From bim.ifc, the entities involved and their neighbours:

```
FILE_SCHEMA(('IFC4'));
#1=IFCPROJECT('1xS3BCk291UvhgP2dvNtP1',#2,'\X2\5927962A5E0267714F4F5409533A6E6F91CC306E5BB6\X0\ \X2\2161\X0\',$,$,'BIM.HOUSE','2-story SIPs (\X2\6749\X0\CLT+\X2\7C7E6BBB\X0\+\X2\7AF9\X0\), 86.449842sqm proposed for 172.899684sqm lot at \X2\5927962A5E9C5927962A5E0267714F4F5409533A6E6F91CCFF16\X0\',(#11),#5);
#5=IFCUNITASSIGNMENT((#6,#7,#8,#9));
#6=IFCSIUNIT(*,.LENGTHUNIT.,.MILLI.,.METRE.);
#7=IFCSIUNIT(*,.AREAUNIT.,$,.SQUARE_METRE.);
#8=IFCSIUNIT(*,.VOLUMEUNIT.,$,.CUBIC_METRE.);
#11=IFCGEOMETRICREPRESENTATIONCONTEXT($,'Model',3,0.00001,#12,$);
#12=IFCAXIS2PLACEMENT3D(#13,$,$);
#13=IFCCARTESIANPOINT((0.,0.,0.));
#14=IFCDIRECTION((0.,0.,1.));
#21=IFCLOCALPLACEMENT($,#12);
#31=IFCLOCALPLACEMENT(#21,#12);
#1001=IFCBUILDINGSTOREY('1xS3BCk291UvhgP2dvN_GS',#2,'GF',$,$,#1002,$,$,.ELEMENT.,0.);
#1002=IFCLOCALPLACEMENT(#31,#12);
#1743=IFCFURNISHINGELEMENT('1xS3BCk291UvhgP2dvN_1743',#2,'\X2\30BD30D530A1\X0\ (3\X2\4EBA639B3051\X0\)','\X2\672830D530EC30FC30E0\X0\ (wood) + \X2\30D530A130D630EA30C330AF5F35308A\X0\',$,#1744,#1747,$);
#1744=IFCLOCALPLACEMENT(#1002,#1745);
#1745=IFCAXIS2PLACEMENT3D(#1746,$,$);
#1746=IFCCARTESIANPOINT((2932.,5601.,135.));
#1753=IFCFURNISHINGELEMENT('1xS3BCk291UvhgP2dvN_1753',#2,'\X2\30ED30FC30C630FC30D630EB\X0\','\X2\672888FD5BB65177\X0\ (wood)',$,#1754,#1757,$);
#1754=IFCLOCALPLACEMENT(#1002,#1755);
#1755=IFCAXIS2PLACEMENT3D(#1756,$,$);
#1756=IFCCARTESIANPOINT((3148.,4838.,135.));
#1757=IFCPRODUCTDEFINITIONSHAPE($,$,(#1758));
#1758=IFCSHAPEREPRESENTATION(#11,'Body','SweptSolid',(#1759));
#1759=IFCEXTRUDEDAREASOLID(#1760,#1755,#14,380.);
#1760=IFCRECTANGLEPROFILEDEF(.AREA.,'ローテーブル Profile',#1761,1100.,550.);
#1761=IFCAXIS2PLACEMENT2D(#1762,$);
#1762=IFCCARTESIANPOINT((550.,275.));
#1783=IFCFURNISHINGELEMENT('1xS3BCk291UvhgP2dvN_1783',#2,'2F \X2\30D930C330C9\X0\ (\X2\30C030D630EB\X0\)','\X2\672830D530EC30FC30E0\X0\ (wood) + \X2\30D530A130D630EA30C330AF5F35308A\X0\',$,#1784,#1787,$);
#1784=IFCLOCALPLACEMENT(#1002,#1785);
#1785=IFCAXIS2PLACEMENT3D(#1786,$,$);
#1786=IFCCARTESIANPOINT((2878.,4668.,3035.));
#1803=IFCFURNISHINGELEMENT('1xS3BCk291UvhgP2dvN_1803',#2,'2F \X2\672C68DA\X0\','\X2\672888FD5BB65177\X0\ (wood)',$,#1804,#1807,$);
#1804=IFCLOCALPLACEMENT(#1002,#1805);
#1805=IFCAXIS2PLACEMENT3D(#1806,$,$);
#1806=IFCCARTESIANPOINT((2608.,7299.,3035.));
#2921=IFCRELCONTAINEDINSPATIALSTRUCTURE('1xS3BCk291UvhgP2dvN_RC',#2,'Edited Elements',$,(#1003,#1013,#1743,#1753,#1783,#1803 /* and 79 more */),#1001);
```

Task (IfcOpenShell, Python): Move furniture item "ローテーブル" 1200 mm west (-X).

```python
import ifcopenshell
import ifcopenshell.api.geometry
import ifcopenshell.util.placement
import ifcopenshell.util.unit

model = ifcopenshell.open("bim.ifc")
unit_scale = ifcopenshell.util.unit.calculate_unit_scale(model)

item = model.by_id(1753)
matrix = ifcopenshell.util.placement.get_local_placement(item.ObjectPlacement)
matrix[0, 3] -= 1.2 / unit_scale
ifcopenshell.api.geometry.edit_object_placement(model, product=item, matrix=matrix, is_si=False)

print(ifcopenshell.util.placement.get_local_placement(item.ObjectPlacement).round(3) + 0.0)

model.write("bim_rev.ifc")
```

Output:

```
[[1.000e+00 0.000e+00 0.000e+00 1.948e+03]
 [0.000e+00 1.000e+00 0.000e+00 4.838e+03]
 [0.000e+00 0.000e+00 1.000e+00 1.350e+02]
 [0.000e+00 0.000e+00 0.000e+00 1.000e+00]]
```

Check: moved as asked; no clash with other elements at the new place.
